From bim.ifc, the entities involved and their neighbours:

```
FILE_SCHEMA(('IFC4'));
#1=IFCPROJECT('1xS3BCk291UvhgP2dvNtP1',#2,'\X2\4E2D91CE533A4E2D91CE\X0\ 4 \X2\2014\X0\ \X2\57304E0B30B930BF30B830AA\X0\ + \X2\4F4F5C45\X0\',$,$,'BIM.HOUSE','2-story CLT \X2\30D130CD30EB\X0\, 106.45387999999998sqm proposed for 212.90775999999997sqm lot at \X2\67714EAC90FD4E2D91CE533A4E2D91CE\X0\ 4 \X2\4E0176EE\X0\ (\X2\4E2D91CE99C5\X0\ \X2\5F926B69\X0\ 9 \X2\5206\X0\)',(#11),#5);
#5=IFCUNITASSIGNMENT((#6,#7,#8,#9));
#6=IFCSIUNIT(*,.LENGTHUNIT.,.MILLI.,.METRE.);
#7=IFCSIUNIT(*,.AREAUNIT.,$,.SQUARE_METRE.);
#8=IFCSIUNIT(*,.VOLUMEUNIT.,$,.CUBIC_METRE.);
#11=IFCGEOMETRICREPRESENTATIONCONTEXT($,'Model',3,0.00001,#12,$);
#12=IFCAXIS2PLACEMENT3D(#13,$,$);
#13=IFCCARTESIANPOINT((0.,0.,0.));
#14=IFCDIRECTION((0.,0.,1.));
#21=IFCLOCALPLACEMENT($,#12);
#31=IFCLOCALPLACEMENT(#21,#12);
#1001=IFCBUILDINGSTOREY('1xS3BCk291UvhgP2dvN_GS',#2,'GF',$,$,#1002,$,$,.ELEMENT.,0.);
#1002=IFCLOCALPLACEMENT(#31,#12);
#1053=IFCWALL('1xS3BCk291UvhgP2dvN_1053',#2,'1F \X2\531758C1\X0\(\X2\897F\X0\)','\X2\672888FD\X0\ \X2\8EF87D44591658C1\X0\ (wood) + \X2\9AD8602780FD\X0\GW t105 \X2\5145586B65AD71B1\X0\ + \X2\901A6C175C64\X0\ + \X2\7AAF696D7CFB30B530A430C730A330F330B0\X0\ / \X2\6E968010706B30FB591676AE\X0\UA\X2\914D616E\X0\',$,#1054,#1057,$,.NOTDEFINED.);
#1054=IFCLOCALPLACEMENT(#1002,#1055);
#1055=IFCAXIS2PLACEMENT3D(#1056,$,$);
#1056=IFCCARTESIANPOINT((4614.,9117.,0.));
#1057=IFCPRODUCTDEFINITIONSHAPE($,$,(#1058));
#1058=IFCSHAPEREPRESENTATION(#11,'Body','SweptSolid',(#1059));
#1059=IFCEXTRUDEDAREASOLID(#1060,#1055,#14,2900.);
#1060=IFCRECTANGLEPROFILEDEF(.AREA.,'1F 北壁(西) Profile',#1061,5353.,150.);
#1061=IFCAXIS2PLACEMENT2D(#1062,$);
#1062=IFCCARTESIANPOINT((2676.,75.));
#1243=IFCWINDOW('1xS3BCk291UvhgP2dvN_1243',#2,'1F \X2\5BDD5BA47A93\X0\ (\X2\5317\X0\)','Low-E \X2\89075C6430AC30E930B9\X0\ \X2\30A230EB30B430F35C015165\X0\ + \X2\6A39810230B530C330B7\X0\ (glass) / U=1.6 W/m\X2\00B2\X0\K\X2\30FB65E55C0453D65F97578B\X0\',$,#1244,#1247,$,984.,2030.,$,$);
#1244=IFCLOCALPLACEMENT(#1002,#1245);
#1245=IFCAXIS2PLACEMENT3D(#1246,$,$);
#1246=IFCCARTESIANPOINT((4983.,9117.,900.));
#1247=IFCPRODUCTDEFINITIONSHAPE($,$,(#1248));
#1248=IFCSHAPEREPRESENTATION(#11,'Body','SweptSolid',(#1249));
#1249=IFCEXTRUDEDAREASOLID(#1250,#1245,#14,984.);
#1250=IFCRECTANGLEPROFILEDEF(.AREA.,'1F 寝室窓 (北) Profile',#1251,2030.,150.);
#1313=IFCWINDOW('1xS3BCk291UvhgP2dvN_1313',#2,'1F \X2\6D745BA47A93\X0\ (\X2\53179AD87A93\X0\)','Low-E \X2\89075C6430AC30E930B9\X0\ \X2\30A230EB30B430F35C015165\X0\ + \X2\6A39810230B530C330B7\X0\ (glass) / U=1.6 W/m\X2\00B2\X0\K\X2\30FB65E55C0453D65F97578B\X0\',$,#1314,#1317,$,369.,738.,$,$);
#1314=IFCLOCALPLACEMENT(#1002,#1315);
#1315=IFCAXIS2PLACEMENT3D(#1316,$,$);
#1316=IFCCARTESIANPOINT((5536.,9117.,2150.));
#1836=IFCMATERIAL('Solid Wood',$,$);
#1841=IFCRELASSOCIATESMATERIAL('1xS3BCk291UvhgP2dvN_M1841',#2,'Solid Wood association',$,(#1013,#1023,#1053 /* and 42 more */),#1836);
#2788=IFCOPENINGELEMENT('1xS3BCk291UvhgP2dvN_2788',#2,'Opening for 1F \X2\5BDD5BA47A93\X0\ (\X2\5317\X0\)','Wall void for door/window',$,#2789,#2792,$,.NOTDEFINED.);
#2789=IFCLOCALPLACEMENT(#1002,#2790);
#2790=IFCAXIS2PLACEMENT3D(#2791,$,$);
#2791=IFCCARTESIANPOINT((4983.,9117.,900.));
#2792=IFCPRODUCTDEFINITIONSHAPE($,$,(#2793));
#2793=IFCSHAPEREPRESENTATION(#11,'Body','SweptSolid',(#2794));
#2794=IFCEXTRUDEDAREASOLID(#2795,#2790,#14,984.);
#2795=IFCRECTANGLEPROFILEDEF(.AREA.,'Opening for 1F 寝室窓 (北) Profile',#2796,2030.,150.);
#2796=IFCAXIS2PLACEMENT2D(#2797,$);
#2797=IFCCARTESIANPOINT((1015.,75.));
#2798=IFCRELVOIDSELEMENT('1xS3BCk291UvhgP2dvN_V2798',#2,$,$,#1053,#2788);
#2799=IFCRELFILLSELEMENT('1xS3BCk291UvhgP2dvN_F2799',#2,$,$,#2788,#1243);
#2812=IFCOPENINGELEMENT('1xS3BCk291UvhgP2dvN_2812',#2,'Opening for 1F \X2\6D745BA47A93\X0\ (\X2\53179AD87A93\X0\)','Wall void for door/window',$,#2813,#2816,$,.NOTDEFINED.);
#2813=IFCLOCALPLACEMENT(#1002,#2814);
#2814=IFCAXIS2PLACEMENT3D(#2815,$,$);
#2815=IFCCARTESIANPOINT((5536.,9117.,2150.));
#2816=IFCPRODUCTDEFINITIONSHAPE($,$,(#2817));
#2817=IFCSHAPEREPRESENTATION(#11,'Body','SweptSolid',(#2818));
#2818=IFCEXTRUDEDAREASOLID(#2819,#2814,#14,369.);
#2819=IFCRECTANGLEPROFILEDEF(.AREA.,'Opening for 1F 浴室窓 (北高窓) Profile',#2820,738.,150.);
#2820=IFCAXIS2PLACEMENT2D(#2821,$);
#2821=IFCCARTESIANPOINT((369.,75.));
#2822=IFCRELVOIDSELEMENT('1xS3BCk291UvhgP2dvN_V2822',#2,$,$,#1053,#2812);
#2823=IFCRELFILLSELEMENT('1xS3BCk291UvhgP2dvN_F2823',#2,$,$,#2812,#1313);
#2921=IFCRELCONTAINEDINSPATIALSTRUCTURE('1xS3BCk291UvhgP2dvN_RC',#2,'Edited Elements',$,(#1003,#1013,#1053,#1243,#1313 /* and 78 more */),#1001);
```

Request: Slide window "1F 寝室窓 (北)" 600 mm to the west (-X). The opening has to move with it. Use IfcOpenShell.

```python
import ifcopenshell
import ifcopenshell.api.geometry
import ifcopenshell.util.placement
import ifcopenshell.util.unit

model = ifcopenshell.open("bim.ifc")
unit_scale = ifcopenshell.util.unit.calculate_unit_scale(model)

window = model.by_guid("1xS3BCk291UvhgP2dvN_1243")
opening = window.FillsVoids[0].RelatingOpeningElement
wall = opening.VoidsElements[0].RelatingBuildingElement

wall_matrix = ifcopenshell.util.placement.get_local_placement(wall.ObjectPlacement)
shift = wall_matrix[:3, 0] * -0.6 / unit_scale
before = ifcopenshell.util.placement.get_local_placement(window.ObjectPlacement)[:3, 3].copy()

# The window is not placed relative to its opening, so move both.
for product in (opening, window):
    matrix = ifcopenshell.util.placement.get_local_placement(product.ObjectPlacement)
    matrix[:3, 3] += shift
    ifcopenshell.api.geometry.edit_object_placement(model, product=product, matrix=matrix, is_si=False)

after = ifcopenshell.util.placement.get_local_placement(window.ObjectPlacement)[:3, 3]
print("window moved by", (after - before).round(3) + 0.0)

model.write("bim_v2.ifc")
```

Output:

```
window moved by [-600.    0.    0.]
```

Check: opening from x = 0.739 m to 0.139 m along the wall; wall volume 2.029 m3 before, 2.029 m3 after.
